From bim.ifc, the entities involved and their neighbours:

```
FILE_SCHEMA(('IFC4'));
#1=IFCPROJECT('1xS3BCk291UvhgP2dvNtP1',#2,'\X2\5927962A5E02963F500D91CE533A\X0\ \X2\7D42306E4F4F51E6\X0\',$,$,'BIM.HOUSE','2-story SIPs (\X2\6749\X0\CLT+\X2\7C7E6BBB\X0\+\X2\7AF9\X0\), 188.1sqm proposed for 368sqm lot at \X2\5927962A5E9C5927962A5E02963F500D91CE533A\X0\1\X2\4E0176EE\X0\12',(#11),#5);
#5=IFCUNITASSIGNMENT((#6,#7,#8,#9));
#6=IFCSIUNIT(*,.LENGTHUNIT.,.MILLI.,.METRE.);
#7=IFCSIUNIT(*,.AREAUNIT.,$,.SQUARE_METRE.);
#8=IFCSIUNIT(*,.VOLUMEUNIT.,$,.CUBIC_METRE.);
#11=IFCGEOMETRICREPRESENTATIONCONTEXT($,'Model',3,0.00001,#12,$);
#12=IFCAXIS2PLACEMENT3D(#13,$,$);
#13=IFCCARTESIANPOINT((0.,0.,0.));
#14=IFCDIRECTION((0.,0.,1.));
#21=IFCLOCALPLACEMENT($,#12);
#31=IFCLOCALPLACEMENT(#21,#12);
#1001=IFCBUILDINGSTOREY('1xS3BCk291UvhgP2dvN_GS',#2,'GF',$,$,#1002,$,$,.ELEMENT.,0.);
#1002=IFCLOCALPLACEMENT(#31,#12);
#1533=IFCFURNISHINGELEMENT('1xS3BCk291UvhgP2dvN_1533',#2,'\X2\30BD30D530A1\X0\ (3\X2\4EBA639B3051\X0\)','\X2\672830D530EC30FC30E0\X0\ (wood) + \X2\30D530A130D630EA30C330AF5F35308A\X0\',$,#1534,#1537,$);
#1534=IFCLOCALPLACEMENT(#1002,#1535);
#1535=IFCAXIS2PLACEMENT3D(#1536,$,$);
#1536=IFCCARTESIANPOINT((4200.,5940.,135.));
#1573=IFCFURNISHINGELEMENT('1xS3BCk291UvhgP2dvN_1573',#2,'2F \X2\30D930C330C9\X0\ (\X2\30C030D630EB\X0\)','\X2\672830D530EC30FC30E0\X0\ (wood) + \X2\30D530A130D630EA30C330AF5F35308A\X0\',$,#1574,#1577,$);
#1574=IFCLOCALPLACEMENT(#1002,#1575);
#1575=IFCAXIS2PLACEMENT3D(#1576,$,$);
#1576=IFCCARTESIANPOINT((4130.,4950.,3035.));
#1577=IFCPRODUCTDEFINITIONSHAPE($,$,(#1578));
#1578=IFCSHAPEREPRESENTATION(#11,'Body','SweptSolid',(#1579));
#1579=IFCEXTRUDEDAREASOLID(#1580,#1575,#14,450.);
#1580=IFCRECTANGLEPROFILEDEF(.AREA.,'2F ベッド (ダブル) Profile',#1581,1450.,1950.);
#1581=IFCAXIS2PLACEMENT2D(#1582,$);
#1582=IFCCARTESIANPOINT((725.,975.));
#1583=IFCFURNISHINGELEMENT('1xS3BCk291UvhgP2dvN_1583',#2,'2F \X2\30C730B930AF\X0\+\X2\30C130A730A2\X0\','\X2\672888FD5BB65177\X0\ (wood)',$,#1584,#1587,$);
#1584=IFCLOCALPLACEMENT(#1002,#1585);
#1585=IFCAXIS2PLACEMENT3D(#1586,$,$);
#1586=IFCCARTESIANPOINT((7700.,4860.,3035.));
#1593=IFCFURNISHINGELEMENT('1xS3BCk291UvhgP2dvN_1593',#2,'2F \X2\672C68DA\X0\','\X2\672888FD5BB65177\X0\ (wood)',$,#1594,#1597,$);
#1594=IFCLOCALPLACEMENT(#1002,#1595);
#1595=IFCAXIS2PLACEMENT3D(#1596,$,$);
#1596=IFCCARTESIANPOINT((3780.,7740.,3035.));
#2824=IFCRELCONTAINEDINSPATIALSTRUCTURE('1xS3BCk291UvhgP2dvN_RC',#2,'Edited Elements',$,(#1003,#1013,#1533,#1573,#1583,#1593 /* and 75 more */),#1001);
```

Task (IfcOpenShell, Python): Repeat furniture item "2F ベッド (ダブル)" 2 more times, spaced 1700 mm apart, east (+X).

```python
import numpy as np
import ifcopenshell
import ifcopenshell.api.geometry
import ifcopenshell.api.root
import ifcopenshell.util.element
import ifcopenshell.util.placement
import ifcopenshell.util.unit

model = ifcopenshell.open("bim.ifc")
unit_scale = ifcopenshell.util.unit.calculate_unit_scale(model)


def reuse_history(source, copy):
    """copy_class also copies each property set's owner history, people and application; keep the originals."""
    for rel in copy.IsDefinedBy:
        if rel.is_a("IfcRelDefinesByProperties") and (history := rel.RelatingPropertyDefinition.OwnerHistory):
            rel.RelatingPropertyDefinition.OwnerHistory = source.OwnerHistory
            ifcopenshell.util.element.remove_deep2(model, history)


source = model.by_id(1573)
base = ifcopenshell.util.placement.get_local_placement(source.ObjectPlacement)
step = np.array([1.0, 0.0, 0.0]) * 1.7 / unit_scale

for i in range(1, 3):
    copy = ifcopenshell.api.root.copy_class(model, product=source)
    copy.Representation = ifcopenshell.util.element.copy_deep(
        model, source.Representation, exclude=["IfcGeometricRepresentationContext", "IfcRepresentationMap"]
    )
    reuse_history(source, copy)
    matrix = base.copy()
    matrix[:3, 3] += i * step
    print("added at", matrix[:3, 3].round(3) + 0.0)
    ifcopenshell.api.geometry.edit_object_placement(model, product=copy, matrix=matrix, is_si=False)

model.write("bim_edited.ifc")
```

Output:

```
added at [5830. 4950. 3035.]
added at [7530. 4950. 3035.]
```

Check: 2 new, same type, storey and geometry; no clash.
